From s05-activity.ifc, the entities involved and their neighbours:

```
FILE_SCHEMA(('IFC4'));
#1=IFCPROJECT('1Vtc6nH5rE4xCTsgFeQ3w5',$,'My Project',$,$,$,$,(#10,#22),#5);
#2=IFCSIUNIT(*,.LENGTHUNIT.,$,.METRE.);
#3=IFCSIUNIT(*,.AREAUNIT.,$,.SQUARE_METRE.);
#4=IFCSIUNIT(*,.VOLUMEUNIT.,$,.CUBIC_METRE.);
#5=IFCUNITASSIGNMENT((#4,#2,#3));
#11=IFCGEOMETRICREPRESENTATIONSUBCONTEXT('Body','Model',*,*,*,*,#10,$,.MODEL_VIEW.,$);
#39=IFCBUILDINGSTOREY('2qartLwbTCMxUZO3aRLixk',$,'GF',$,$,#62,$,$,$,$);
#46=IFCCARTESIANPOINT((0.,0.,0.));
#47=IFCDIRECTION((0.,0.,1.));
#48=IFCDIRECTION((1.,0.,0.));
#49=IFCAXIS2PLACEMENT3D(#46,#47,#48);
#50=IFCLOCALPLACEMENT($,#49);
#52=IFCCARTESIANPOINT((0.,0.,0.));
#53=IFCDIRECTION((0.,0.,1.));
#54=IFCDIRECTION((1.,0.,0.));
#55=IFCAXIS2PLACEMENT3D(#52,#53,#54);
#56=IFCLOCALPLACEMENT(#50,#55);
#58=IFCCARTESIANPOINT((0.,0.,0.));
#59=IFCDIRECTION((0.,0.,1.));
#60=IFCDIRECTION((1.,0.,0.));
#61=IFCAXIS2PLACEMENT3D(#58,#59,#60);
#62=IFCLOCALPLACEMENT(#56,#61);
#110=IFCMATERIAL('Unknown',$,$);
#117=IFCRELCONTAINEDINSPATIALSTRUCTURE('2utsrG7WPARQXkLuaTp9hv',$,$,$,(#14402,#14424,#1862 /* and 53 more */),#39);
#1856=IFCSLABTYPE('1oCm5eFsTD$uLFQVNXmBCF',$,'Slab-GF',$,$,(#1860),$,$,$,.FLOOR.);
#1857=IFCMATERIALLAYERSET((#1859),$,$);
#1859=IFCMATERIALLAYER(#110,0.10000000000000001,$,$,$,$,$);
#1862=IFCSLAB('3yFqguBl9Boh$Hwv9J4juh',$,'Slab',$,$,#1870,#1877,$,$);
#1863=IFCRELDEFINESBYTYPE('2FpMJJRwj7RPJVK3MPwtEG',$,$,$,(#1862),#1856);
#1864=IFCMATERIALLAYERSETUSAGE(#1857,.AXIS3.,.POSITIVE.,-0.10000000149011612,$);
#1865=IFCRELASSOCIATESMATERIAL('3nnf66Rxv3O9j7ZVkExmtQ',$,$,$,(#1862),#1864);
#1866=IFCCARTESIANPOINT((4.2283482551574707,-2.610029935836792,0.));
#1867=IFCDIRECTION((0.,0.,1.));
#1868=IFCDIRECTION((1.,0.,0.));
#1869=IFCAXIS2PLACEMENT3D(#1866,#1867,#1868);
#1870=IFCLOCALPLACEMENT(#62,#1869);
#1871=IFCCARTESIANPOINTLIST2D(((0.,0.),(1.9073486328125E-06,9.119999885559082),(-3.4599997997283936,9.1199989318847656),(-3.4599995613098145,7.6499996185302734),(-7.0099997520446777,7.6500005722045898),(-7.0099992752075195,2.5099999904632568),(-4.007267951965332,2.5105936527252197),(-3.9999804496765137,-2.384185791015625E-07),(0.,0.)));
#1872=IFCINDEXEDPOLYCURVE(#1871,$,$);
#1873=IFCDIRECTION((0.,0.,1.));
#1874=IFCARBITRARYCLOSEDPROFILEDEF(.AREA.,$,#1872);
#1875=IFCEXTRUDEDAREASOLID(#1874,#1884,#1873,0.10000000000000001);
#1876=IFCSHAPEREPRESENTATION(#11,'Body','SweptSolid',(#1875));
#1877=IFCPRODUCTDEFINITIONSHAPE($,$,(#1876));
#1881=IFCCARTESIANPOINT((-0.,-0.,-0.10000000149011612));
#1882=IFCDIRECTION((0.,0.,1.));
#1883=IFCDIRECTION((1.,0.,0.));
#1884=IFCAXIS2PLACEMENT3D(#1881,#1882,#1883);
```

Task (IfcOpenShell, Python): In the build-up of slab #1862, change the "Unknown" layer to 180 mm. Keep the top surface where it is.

```python
import ifcopenshell
import ifcopenshell.util.element
import ifcopenshell.util.representation
import ifcopenshell.util.unit

model = ifcopenshell.open("s05-activity.ifc")
unit_scale = ifcopenshell.util.unit.calculate_unit_scale(model)

layer_set = model.by_id(1857)
layer = next(l for l in layer_set.MaterialLayers if l.Material and l.Material.Name == "Unknown")
change = 0.18 / unit_scale - layer.LayerThickness
layer.LayerThickness += change

# Geometry does not follow the layer set by itself.
slabs = [e for e in ifcopenshell.util.element.get_elements_by_material(model, layer_set) if e.is_a("IfcSlab")]
for slab in sorted(slabs, key=lambda e: e.id()):
    body = ifcopenshell.util.representation.get_representation(slab, "Model", "Body")
    solid = body.Items[0]
    old_depth = solid.Depth
    solid.Depth += change
    # Extruded upwards: lower the start of the extrusion so the top stays.
    x, y, z = solid.Position.Location.Coordinates
    solid.Position.Location = model.createIfcCartesianPoint((x, y, z - change))
    print(slab.id(), f"{old_depth:g} -> {solid.Depth:g}")

# The layers are counted up from the underside, which has moved.
for usage in {ifcopenshell.util.element.get_material(slab) for slab in slabs}:
    usage.OffsetFromReferenceLine -= change

model.write("s05-activity_rev.ifc")
```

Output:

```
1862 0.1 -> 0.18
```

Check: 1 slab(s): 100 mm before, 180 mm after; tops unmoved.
